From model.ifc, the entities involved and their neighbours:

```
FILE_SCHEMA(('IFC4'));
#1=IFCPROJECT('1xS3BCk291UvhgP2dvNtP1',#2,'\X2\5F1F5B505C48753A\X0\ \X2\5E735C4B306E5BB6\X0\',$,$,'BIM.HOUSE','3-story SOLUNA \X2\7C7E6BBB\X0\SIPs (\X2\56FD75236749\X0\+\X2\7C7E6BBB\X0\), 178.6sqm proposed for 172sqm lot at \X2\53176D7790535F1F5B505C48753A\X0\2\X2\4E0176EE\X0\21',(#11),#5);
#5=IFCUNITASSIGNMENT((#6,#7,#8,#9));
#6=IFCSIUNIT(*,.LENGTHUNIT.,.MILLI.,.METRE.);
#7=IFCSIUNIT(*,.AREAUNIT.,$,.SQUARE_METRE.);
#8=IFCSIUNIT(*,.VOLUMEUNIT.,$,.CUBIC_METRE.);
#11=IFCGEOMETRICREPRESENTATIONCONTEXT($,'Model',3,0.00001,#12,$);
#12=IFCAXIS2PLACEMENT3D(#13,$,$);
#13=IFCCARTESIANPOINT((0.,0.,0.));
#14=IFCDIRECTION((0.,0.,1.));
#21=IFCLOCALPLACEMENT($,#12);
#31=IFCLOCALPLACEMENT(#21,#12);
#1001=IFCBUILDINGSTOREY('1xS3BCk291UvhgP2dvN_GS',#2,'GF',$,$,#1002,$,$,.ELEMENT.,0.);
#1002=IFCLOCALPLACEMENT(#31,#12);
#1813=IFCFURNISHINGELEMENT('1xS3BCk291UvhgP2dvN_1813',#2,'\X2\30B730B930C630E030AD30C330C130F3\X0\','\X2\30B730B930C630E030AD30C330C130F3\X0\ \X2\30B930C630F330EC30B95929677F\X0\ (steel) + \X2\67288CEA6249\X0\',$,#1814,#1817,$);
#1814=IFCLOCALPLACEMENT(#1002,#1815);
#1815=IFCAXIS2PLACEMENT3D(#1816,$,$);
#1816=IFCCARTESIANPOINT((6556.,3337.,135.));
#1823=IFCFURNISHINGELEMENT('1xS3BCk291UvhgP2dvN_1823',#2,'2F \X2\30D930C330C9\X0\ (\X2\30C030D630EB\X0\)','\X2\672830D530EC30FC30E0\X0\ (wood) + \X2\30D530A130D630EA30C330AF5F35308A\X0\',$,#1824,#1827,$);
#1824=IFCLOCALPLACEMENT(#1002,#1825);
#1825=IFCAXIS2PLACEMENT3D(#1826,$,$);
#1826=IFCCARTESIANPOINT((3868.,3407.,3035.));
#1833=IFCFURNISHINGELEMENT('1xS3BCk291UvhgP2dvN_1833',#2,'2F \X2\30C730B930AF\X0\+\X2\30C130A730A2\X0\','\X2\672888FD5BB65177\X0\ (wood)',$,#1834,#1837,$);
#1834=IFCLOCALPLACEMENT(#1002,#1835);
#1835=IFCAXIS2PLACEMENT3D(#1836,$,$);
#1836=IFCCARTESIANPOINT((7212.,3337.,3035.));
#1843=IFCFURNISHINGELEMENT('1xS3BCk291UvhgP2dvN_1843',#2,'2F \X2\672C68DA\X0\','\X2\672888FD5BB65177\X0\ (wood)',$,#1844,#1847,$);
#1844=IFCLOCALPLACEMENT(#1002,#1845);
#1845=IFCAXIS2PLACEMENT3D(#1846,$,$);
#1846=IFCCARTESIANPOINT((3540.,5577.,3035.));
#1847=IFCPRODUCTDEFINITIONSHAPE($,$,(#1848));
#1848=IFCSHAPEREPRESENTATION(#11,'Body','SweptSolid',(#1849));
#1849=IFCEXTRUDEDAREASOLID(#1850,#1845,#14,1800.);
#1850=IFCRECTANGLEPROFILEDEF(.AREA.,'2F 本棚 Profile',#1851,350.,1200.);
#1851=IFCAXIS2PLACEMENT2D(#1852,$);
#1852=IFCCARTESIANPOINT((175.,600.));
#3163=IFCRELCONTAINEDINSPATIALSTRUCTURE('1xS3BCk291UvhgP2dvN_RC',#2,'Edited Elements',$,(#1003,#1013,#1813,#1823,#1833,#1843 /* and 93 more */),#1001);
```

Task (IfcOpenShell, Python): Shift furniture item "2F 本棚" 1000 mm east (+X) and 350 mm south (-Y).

```python
import ifcopenshell
import ifcopenshell.api.geometry
import ifcopenshell.util.placement

model = ifcopenshell.open("model.ifc")

item = model.by_guid("1xS3BCk291UvhgP2dvN_1843")
matrix = ifcopenshell.util.placement.get_local_placement(item.ObjectPlacement)
matrix[0, 3] += 1000.0
matrix[1, 3] -= 350.0
ifcopenshell.api.geometry.edit_object_placement(model, product=item, matrix=matrix, is_si=False)

print(ifcopenshell.util.placement.get_local_placement(item.ObjectPlacement).round(3) + 0.0)

model.write("model_rev.ifc")
```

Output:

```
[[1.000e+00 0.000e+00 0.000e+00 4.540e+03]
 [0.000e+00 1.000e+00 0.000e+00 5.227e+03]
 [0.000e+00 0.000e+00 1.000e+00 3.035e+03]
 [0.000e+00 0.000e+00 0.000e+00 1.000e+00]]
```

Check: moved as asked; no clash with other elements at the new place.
